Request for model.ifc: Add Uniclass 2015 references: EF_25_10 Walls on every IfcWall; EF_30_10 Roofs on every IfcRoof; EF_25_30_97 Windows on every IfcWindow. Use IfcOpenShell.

First a look at what the model holds.

```python
import ifcopenshell

model = ifcopenshell.open("model.ifc")
print(model.schema)
print("classifications:", [c.Name for c in model.by_type("IfcClassification")])
for ifc_class in ("IfcDoor", "IfcRoof", "IfcStair", "IfcWall", "IfcWindow"):
    print(ifc_class, len(model.by_type(ifc_class)))
```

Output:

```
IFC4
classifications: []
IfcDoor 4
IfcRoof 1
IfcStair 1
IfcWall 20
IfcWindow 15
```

```python
import ifcopenshell
import ifcopenshell.api.classification

model = ifcopenshell.open("model.ifc")

system = ifcopenshell.api.classification.add_classification(model, classification="Uniclass 2015")

codes = {
    "IfcWall": ("EF_25_10", "Walls"),
    "IfcRoof": ("EF_30_10", "Roofs"),
    "IfcWindow": ("EF_25_30_97", "Windows"),
}
for ifc_class, (code, name) in codes.items():
    products = model.by_type(ifc_class)
    ifcopenshell.api.classification.add_reference(
        model, products=products, classification=system, identification=code, name=name
    )
    print(code, len(products))

model.write("model_v2.ifc")
```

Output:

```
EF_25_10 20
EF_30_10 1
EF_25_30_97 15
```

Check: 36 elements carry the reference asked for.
